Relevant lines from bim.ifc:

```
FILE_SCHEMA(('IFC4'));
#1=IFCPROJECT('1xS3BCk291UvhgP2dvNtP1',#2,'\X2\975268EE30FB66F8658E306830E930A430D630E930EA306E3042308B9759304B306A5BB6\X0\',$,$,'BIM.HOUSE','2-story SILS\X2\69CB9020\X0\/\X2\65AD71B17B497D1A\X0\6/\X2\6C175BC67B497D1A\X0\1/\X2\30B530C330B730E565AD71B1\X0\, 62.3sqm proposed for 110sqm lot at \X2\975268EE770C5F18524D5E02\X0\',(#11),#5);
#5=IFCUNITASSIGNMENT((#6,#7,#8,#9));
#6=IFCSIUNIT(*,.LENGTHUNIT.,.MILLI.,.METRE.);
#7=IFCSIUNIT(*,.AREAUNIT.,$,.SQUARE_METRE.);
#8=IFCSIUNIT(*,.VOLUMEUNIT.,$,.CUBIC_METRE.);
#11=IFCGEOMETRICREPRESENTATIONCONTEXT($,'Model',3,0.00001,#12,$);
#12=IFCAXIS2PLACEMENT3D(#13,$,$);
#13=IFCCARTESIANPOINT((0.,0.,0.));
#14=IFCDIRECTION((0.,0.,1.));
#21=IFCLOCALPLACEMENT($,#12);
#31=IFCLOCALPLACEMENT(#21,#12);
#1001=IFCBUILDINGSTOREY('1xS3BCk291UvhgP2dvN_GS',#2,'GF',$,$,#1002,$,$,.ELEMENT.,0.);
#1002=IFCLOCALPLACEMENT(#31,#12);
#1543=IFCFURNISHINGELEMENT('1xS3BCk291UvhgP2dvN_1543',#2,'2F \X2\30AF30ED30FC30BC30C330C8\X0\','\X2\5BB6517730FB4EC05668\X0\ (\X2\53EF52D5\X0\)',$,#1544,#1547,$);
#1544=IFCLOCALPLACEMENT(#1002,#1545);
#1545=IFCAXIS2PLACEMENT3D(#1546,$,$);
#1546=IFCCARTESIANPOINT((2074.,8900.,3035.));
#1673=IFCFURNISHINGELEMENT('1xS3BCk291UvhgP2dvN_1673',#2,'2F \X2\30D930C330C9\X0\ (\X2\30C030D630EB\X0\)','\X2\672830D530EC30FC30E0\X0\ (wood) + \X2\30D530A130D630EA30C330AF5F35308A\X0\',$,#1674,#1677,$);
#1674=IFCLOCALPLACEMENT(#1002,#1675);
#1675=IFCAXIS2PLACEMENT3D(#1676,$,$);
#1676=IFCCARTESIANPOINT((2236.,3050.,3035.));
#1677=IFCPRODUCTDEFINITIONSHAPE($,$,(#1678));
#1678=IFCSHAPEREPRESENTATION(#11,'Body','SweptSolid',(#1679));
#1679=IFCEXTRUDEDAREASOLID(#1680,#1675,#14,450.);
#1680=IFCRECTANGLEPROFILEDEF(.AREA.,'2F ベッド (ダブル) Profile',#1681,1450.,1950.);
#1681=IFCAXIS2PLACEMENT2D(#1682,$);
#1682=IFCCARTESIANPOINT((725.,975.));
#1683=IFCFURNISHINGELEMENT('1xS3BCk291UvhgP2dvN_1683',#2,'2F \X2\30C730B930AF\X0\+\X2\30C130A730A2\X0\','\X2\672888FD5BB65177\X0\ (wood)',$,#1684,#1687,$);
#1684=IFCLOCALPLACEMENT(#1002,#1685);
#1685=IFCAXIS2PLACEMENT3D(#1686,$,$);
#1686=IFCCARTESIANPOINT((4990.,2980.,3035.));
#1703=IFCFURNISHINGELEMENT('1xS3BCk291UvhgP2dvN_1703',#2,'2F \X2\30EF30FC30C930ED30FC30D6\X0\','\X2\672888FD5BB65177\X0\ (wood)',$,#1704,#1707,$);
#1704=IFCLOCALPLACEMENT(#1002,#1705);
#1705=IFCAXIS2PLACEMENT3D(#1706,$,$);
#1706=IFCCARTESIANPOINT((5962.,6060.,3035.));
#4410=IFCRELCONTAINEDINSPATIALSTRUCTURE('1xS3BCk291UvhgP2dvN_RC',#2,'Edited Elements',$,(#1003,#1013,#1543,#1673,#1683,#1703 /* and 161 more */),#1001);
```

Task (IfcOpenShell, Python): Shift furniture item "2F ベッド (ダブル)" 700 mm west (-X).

```python
import ifcopenshell
import ifcopenshell.api.geometry
import ifcopenshell.util.placement
import ifcopenshell.util.unit

model = ifcopenshell.open("bim.ifc")
unit_scale = ifcopenshell.util.unit.calculate_unit_scale(model)

item = model.by_guid("1xS3BCk291UvhgP2dvN_1673")
matrix = ifcopenshell.util.placement.get_local_placement(item.ObjectPlacement)
matrix[0, 3] -= 0.7 / unit_scale
ifcopenshell.api.geometry.edit_object_placement(model, product=item, matrix=matrix, is_si=False)

print(ifcopenshell.util.placement.get_local_placement(item.ObjectPlacement).round(3) + 0.0)

model.write("bim_updated.ifc")
```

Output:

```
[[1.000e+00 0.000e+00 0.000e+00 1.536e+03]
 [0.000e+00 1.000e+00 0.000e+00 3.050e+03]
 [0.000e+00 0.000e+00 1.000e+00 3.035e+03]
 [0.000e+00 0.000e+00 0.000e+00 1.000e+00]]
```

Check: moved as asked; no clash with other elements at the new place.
